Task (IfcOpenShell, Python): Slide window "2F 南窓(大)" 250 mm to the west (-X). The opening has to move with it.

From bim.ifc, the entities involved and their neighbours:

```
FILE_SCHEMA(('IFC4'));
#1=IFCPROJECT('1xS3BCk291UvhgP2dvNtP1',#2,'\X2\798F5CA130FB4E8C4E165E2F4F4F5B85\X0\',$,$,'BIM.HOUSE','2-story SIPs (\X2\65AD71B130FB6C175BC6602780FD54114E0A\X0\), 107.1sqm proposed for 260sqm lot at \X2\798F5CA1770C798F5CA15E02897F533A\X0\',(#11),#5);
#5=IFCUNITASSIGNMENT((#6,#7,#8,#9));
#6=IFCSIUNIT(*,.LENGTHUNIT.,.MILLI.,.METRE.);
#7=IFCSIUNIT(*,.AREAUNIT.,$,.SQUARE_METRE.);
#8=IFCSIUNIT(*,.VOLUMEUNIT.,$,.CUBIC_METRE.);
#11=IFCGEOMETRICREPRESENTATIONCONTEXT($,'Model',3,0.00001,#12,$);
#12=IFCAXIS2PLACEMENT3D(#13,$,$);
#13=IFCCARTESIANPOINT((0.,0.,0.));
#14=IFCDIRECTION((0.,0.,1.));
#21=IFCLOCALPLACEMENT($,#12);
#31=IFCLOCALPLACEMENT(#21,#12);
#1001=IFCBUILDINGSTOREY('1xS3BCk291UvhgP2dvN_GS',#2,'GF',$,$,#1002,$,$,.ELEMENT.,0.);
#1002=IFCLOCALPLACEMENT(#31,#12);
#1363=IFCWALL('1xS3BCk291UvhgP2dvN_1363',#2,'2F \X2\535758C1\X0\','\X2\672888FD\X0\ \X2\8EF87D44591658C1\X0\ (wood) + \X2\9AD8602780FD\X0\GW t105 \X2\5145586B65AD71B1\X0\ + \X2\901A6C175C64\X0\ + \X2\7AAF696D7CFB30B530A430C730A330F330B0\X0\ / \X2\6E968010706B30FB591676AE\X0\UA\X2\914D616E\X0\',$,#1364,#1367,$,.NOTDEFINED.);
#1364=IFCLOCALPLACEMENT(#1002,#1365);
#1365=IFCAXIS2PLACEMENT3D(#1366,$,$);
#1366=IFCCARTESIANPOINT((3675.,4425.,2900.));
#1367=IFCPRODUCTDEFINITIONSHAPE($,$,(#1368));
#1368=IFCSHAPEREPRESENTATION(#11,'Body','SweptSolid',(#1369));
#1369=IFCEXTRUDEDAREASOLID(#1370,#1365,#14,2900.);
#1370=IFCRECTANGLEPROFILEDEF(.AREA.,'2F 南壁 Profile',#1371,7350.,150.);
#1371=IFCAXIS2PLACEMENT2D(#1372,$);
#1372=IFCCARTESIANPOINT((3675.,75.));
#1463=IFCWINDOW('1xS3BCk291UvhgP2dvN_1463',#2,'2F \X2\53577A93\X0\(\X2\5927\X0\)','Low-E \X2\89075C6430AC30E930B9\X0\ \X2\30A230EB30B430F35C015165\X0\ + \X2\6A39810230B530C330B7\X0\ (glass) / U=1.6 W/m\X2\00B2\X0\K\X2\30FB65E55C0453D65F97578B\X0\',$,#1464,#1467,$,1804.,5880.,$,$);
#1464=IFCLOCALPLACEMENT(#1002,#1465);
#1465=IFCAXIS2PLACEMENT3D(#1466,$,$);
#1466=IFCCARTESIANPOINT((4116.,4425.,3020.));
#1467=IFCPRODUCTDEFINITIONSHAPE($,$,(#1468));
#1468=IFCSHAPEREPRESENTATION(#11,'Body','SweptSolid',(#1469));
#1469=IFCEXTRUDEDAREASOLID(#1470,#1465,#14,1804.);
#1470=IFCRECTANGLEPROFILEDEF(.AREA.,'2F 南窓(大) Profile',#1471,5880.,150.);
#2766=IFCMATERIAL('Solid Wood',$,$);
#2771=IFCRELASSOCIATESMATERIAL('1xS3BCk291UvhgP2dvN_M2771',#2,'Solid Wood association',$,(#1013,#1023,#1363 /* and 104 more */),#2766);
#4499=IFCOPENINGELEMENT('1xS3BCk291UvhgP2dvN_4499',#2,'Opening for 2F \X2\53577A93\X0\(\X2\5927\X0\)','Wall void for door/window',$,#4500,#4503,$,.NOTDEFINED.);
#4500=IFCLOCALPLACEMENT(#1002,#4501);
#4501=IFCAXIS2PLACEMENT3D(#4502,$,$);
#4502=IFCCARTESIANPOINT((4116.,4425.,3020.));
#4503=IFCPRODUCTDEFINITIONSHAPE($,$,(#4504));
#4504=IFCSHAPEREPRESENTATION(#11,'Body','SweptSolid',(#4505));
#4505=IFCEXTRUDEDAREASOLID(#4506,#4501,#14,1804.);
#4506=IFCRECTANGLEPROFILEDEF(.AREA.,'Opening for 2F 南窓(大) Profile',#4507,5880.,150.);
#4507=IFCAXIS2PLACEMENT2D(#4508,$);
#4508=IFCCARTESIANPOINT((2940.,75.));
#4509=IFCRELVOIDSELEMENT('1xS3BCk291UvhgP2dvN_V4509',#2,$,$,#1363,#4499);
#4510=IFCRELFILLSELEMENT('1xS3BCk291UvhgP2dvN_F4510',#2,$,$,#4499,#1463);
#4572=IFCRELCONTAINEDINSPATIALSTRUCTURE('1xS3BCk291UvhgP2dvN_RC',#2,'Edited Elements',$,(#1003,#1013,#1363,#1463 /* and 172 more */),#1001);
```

```python
import ifcopenshell
import ifcopenshell.api.geometry
import ifcopenshell.util.placement
import ifcopenshell.util.unit

model = ifcopenshell.open("bim.ifc")
unit_scale = ifcopenshell.util.unit.calculate_unit_scale(model)

window = model.by_guid("1xS3BCk291UvhgP2dvN_1463")
opening = window.FillsVoids[0].RelatingOpeningElement
wall = opening.VoidsElements[0].RelatingBuildingElement

wall_matrix = ifcopenshell.util.placement.get_local_placement(wall.ObjectPlacement)
shift = wall_matrix[:3, 0] * -0.25 / unit_scale
before = ifcopenshell.util.placement.get_local_placement(window.ObjectPlacement)[:3, 3].copy()

# The window is not placed relative to its opening, so move both.
for product in (opening, window):
    matrix = ifcopenshell.util.placement.get_local_placement(product.ObjectPlacement)
    matrix[:3, 3] += shift
    ifcopenshell.api.geometry.edit_object_placement(model, product=product, matrix=matrix, is_si=False)

after = ifcopenshell.util.placement.get_local_placement(window.ObjectPlacement)[:3, 3]
print("window moved by", (after - before).round(3) + 0.0)

model.write("bim_edited.ifc")
```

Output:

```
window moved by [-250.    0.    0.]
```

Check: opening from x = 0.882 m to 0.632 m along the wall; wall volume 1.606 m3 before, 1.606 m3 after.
